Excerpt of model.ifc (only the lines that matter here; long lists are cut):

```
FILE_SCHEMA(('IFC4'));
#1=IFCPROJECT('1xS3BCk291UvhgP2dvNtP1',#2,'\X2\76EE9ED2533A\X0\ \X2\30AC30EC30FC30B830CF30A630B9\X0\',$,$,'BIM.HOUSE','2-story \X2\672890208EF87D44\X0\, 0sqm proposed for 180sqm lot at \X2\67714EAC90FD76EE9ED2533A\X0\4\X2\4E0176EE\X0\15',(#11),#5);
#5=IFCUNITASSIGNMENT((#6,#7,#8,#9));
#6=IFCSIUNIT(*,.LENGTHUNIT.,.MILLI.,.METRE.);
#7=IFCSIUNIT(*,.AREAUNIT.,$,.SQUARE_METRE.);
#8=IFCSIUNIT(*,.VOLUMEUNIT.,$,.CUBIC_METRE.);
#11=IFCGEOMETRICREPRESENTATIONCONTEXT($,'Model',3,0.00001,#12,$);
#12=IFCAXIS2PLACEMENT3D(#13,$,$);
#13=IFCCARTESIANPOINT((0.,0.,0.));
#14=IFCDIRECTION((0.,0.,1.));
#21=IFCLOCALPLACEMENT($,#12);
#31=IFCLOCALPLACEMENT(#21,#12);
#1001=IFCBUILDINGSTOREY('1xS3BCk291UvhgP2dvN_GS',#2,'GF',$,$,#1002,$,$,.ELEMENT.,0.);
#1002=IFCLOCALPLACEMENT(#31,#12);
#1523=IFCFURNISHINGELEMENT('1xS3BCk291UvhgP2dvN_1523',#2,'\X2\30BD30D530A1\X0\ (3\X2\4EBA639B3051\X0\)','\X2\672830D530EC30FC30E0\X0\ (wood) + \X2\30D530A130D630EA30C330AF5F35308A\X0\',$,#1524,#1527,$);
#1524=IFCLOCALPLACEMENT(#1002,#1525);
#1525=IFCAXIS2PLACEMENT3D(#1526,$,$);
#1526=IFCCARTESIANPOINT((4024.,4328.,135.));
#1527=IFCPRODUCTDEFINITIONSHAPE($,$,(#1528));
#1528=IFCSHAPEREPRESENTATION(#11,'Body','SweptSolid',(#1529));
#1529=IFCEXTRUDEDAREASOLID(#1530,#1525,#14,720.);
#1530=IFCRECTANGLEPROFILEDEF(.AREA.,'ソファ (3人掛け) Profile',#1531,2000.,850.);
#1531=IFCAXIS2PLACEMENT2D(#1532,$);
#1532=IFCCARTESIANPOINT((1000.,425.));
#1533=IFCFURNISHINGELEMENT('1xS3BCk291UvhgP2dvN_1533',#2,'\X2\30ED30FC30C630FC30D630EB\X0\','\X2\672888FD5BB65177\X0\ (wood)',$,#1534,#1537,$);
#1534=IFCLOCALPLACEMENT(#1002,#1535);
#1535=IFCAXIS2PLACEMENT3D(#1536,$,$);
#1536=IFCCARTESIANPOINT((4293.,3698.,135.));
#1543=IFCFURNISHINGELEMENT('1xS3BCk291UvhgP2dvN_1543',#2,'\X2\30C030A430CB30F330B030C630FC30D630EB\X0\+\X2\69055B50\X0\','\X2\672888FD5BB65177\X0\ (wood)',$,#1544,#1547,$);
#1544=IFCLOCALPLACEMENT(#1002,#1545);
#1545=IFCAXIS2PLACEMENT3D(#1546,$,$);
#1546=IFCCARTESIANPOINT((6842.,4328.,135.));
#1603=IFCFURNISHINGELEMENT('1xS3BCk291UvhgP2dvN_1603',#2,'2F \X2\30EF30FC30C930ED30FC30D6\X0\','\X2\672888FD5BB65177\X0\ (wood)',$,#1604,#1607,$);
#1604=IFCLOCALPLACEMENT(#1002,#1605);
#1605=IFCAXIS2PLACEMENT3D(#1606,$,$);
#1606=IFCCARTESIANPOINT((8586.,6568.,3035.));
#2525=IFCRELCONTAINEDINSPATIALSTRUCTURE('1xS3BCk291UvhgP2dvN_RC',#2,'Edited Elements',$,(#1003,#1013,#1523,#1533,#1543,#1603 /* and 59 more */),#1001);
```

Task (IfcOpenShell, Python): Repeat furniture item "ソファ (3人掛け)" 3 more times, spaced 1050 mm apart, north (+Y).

```python
import numpy as np
import ifcopenshell
import ifcopenshell.api.geometry
import ifcopenshell.api.root
import ifcopenshell.util.element
import ifcopenshell.util.placement
import ifcopenshell.util.unit

model = ifcopenshell.open("model.ifc")
unit_scale = ifcopenshell.util.unit.calculate_unit_scale(model)


def reuse_history(source, copy):
    """copy_class also copies each property set's owner history, people and application; keep the originals."""
    for rel in copy.IsDefinedBy:
        if rel.is_a("IfcRelDefinesByProperties") and (history := rel.RelatingPropertyDefinition.OwnerHistory):
            rel.RelatingPropertyDefinition.OwnerHistory = source.OwnerHistory
            ifcopenshell.util.element.remove_deep2(model, history)


source = model.by_guid("1xS3BCk291UvhgP2dvN_1523")
base = ifcopenshell.util.placement.get_local_placement(source.ObjectPlacement)
step = np.array([0.0, 1.0, 0.0]) * 1.05 / unit_scale

for i in range(1, 4):
    copy = ifcopenshell.api.root.copy_class(model, product=source)
    copy.Representation = ifcopenshell.util.element.copy_deep(
        model, source.Representation, exclude=["IfcGeometricRepresentationContext", "IfcRepresentationMap"]
    )
    reuse_history(source, copy)
    matrix = base.copy()
    matrix[:3, 3] += i * step
    print("added at", matrix[:3, 3].round(3) + 0.0)
    ifcopenshell.api.geometry.edit_object_placement(model, product=copy, matrix=matrix, is_si=False)

model.write("model_rev.ifc")
```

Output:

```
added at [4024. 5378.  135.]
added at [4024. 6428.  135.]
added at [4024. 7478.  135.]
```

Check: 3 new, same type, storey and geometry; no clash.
